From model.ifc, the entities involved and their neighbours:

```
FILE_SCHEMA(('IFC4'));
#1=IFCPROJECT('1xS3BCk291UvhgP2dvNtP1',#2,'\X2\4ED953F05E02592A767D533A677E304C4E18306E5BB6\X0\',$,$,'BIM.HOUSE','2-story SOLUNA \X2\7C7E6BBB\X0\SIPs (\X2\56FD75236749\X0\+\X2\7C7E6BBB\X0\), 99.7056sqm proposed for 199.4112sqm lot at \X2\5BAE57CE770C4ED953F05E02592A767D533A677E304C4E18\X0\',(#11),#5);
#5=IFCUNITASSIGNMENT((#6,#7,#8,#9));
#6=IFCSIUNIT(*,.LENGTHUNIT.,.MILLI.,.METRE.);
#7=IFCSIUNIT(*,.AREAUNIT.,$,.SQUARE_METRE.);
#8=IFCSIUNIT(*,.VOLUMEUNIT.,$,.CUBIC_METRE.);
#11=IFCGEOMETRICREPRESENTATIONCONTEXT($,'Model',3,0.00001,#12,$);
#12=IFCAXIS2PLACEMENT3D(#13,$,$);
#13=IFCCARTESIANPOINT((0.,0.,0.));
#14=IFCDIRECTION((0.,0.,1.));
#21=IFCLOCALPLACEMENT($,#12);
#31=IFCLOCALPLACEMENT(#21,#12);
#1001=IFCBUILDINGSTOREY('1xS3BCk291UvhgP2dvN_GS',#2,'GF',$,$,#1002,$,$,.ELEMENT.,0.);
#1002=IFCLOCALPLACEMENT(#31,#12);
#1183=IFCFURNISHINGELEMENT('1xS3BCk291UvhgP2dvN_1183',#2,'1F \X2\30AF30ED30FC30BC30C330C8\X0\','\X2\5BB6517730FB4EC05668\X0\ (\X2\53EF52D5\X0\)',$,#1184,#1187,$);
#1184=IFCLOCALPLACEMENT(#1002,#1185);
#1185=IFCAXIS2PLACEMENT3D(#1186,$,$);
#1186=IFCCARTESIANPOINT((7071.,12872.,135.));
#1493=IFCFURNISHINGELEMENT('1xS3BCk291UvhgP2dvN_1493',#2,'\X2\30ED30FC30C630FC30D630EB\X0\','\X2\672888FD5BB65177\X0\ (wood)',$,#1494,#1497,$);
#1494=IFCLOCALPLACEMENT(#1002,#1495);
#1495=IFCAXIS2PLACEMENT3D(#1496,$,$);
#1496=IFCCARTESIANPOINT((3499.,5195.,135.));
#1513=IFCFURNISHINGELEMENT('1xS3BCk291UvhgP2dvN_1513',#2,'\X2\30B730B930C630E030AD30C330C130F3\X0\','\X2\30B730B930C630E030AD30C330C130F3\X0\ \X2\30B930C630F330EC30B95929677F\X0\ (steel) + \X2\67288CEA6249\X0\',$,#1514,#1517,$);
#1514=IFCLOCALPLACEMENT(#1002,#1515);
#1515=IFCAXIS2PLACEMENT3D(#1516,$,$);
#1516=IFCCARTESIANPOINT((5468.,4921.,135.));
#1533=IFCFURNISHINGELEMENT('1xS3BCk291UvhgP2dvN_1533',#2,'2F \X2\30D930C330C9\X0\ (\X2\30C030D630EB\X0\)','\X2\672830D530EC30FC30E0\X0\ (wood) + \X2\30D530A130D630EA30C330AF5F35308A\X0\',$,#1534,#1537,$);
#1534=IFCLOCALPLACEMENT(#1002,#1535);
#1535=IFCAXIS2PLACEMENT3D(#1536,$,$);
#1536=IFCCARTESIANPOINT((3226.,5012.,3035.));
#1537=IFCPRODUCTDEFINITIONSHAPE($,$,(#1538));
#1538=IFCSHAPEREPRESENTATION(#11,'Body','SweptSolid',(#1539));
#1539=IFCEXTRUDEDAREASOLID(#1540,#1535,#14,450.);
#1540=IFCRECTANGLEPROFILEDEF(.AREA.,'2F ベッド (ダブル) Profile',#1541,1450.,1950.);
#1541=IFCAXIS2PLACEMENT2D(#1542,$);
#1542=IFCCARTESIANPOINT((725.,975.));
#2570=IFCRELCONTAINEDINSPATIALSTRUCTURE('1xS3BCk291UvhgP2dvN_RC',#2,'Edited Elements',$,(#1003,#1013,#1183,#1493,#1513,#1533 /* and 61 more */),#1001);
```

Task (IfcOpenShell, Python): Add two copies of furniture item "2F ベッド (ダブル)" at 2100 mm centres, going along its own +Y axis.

```python
import ifcopenshell
import ifcopenshell.api.geometry
import ifcopenshell.api.root
import ifcopenshell.util.element
import ifcopenshell.util.placement
import ifcopenshell.util.unit

model = ifcopenshell.open("model.ifc")
unit_scale = ifcopenshell.util.unit.calculate_unit_scale(model)


def reuse_history(source, copy):
    """copy_class also copies each property set's owner history, people and application; keep the originals."""
    for rel in copy.IsDefinedBy:
        if rel.is_a("IfcRelDefinesByProperties") and (history := rel.RelatingPropertyDefinition.OwnerHistory):
            rel.RelatingPropertyDefinition.OwnerHistory = source.OwnerHistory
            ifcopenshell.util.element.remove_deep2(model, history)


source = model.by_id(1533)
base = ifcopenshell.util.placement.get_local_placement(source.ObjectPlacement)
step = base[:3, 1] * 2.1 / unit_scale

for i in range(1, 3):
    copy = ifcopenshell.api.root.copy_class(model, product=source)
    copy.Representation = ifcopenshell.util.element.copy_deep(
        model, source.Representation, exclude=["IfcGeometricRepresentationContext", "IfcRepresentationMap"]
    )
    reuse_history(source, copy)
    matrix = base.copy()
    matrix[:3, 3] += i * step
    print("added at", matrix[:3, 3].round(3) + 0.0)
    ifcopenshell.api.geometry.edit_object_placement(model, product=copy, matrix=matrix, is_si=False)

model.write("model_edited.ifc")
```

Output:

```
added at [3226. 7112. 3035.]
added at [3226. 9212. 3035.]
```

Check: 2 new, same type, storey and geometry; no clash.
